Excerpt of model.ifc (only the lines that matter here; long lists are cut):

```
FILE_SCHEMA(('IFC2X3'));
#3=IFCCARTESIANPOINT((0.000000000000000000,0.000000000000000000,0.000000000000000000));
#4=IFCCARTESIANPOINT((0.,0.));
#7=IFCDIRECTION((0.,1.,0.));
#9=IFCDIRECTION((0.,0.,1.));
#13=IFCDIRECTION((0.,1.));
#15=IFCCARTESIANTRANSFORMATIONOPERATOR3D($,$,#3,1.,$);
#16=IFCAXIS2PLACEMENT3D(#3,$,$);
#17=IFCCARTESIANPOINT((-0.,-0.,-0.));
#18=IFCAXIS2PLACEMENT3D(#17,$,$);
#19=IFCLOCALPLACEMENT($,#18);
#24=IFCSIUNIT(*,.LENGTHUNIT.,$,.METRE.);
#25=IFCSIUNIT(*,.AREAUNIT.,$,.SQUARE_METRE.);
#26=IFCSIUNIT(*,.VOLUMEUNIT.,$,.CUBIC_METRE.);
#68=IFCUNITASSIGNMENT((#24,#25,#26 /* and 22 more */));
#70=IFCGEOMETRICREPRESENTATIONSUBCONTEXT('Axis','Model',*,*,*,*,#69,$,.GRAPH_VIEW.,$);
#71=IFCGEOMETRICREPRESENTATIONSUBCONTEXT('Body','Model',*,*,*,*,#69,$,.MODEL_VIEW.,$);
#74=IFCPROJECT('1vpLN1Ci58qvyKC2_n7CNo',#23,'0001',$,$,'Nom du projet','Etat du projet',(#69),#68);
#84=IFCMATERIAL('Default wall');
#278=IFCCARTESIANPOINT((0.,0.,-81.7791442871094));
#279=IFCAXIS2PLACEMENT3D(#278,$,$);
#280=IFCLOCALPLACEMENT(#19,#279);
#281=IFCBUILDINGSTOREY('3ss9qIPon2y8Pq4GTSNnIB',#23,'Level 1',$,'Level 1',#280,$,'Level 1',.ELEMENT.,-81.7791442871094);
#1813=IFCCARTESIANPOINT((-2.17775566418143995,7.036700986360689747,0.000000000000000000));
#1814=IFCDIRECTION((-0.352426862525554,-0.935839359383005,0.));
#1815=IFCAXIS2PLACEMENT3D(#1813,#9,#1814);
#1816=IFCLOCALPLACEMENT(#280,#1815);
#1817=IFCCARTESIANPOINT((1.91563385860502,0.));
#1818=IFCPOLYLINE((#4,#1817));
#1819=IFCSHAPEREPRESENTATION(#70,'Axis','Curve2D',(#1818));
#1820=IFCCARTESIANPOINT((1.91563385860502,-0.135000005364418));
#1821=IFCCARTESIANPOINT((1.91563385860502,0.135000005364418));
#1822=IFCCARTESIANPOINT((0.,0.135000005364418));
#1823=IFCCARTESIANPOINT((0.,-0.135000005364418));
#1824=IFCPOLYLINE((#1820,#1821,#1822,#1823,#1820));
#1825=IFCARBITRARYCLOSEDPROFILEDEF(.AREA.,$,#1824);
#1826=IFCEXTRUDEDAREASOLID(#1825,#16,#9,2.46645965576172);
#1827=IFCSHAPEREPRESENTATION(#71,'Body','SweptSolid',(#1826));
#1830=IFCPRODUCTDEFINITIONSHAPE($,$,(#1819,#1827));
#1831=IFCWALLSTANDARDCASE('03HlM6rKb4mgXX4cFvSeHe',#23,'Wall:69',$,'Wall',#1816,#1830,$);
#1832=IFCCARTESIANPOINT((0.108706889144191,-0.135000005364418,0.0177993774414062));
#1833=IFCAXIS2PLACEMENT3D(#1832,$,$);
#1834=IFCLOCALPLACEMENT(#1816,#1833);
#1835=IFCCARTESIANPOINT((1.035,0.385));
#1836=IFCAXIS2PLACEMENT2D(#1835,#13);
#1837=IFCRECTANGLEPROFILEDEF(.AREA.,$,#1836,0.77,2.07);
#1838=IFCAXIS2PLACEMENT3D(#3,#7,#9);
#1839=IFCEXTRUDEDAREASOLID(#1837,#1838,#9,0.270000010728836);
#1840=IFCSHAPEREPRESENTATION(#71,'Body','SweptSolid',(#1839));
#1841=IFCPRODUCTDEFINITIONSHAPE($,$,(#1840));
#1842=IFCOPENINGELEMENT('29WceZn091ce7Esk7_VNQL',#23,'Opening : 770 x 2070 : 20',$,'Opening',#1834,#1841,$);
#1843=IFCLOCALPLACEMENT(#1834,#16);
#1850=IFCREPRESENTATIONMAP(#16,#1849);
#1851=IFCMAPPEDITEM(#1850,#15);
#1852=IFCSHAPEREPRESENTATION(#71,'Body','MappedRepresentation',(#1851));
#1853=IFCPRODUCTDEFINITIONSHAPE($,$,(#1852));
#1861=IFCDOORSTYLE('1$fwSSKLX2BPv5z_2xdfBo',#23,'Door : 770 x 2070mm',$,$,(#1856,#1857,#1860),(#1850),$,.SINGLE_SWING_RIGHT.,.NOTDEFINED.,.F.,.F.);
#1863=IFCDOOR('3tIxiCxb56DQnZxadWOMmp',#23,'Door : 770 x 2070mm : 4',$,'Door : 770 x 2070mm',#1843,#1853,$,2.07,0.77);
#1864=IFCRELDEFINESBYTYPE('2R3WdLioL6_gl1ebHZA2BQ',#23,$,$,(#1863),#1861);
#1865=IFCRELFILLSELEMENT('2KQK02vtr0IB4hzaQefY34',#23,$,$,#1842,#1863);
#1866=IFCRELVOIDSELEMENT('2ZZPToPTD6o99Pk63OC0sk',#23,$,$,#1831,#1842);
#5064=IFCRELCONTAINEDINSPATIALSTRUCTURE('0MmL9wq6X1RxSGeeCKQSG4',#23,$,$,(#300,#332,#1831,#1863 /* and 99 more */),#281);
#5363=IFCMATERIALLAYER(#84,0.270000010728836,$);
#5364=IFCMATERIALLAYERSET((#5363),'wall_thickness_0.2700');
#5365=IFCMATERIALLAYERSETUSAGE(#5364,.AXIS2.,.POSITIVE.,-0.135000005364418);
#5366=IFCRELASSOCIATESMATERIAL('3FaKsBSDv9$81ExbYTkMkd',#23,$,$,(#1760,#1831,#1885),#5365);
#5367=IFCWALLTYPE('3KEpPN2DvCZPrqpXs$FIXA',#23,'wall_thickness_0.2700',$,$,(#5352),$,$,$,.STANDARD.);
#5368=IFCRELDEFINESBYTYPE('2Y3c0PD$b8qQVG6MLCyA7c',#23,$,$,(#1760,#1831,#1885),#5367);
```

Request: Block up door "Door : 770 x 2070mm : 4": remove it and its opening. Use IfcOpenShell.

```python
import ifcopenshell
import ifcopenshell.api.feature
import ifcopenshell.api.root
import ifcopenshell.geom
import ifcopenshell.util.shape

model = ifcopenshell.open("model.ifc")
settings = ifcopenshell.geom.settings()


def volume(element):
    """Net volume in cubic metres, openings subtracted."""
    shape = ifcopenshell.geom.create_shape(settings, element)
    return ifcopenshell.util.shape.get_volume(shape.geometry)


door = model.by_guid("3tIxiCxb56DQnZxadWOMmp")
opening = door.FillsVoids[0].RelatingOpeningElement
wall = opening.VoidsElements[0].RelatingBuildingElement
before = volume(wall)

ifcopenshell.api.root.remove_product(model, product=door)
ifcopenshell.api.feature.remove_feature(model, feature=opening)

after = volume(wall)

print(f"wall volume {before:.3f} -> {after:.3f} m3")

model.write("model_edited.ifc")
```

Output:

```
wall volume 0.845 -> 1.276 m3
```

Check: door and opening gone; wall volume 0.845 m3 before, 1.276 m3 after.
